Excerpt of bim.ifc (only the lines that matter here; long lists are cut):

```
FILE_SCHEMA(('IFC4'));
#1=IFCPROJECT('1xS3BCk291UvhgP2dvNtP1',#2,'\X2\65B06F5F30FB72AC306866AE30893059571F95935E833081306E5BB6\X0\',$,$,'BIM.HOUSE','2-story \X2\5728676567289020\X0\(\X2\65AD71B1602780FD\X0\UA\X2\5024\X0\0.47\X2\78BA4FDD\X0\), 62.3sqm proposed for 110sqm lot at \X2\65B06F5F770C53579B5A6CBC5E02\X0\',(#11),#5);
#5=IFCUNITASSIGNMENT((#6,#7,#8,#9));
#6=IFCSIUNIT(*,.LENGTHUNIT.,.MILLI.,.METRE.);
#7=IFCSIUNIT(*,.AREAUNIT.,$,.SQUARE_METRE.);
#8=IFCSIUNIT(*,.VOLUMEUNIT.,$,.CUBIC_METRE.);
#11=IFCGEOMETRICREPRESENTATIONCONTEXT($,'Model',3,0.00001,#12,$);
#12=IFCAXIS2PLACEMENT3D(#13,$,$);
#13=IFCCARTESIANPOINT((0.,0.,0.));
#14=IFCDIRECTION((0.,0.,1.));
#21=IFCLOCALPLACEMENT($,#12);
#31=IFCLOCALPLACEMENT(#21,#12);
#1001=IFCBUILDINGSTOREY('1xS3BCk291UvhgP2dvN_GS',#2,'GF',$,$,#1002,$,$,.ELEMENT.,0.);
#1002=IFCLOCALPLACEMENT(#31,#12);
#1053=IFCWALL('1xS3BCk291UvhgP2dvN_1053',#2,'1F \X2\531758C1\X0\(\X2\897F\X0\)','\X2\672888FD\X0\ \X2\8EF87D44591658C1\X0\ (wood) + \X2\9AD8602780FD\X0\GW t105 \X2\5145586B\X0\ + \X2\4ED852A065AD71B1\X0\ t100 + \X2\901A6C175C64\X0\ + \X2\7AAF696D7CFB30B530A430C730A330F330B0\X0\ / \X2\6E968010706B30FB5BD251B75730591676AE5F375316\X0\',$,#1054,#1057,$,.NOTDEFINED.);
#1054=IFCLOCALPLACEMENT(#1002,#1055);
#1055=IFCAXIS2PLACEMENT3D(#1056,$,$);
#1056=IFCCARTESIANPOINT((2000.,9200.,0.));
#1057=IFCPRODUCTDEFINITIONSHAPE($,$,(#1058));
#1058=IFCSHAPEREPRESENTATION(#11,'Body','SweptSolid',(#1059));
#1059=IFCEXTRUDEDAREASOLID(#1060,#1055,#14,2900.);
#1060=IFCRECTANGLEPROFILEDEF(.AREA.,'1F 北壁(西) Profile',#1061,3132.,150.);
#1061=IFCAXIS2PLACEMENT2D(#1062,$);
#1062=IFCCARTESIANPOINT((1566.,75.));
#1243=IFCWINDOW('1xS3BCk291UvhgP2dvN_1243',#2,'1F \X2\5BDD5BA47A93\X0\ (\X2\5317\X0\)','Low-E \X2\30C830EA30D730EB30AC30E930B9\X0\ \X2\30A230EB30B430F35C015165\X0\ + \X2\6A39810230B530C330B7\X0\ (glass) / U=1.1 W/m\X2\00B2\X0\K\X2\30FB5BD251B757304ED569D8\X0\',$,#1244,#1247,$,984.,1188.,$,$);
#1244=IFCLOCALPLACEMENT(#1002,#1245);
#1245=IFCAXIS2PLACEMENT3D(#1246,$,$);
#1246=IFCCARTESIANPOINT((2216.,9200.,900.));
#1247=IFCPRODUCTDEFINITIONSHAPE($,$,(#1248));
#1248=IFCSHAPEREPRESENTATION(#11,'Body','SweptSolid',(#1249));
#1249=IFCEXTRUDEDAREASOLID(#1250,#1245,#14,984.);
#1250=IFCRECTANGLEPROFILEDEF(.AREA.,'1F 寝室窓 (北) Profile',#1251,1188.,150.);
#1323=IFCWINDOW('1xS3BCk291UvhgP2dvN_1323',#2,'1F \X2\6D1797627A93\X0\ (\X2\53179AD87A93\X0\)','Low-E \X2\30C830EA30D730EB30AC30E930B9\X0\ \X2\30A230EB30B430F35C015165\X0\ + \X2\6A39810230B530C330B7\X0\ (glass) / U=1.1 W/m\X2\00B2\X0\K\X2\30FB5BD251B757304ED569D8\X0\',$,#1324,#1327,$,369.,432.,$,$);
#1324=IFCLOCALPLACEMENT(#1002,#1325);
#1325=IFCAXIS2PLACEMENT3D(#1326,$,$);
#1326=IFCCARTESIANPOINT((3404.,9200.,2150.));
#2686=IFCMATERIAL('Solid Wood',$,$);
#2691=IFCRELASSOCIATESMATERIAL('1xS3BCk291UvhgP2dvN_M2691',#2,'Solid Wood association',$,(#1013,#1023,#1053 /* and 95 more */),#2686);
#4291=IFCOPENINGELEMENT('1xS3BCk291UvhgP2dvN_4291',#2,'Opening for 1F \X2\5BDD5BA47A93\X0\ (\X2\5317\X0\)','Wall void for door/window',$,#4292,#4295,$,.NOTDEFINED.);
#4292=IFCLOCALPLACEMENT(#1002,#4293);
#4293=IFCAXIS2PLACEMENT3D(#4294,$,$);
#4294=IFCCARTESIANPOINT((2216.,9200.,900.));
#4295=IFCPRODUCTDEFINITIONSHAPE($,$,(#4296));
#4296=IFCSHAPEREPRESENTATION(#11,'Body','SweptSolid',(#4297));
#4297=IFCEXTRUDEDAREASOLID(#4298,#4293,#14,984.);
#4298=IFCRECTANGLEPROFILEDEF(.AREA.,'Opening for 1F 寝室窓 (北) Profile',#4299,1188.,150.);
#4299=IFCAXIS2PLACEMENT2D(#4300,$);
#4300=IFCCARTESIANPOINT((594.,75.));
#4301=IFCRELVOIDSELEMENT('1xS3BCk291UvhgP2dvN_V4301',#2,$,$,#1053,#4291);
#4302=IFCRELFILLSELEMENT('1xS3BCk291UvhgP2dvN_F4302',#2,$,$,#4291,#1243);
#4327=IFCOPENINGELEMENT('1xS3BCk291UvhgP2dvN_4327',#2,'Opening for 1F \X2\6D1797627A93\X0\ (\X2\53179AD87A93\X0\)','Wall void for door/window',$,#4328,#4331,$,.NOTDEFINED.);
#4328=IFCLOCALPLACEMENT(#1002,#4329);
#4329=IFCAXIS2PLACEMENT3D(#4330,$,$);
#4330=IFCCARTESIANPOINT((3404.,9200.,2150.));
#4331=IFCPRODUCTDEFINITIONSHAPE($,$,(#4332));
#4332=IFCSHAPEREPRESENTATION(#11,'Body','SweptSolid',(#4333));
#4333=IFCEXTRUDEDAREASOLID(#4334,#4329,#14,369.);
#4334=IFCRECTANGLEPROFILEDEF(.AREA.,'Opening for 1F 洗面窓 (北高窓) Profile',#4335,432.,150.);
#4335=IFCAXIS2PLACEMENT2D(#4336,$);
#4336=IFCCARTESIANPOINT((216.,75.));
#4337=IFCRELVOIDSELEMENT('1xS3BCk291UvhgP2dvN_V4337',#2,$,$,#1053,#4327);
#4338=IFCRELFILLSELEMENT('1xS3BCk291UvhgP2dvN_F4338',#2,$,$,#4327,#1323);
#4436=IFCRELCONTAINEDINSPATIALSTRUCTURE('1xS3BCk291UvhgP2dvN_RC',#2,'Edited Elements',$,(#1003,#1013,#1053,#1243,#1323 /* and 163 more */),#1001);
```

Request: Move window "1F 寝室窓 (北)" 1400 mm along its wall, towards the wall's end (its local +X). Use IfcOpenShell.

```python
import ifcopenshell
import ifcopenshell.api.geometry
import ifcopenshell.util.placement

model = ifcopenshell.open("bim.ifc")

window = model.by_guid("1xS3BCk291UvhgP2dvN_1243")
opening = window.FillsVoids[0].RelatingOpeningElement
wall = opening.VoidsElements[0].RelatingBuildingElement

wall_matrix = ifcopenshell.util.placement.get_local_placement(wall.ObjectPlacement)
shift = wall_matrix[:3, 0] * 1400.0
before = ifcopenshell.util.placement.get_local_placement(window.ObjectPlacement)[:3, 3].copy()

# The window is not placed relative to its opening, so move both.
for product in (opening, window):
    matrix = ifcopenshell.util.placement.get_local_placement(product.ObjectPlacement)
    matrix[:3, 3] += shift
    ifcopenshell.api.geometry.edit_object_placement(model, product=product, matrix=matrix, is_si=False)

after = ifcopenshell.util.placement.get_local_placement(window.ObjectPlacement)[:3, 3]
print("window moved by", (after - before).round(3) + 0.0)

model.write("bim_rev.ifc")
```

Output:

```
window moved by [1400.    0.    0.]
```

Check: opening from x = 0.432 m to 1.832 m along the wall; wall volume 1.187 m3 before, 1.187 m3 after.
